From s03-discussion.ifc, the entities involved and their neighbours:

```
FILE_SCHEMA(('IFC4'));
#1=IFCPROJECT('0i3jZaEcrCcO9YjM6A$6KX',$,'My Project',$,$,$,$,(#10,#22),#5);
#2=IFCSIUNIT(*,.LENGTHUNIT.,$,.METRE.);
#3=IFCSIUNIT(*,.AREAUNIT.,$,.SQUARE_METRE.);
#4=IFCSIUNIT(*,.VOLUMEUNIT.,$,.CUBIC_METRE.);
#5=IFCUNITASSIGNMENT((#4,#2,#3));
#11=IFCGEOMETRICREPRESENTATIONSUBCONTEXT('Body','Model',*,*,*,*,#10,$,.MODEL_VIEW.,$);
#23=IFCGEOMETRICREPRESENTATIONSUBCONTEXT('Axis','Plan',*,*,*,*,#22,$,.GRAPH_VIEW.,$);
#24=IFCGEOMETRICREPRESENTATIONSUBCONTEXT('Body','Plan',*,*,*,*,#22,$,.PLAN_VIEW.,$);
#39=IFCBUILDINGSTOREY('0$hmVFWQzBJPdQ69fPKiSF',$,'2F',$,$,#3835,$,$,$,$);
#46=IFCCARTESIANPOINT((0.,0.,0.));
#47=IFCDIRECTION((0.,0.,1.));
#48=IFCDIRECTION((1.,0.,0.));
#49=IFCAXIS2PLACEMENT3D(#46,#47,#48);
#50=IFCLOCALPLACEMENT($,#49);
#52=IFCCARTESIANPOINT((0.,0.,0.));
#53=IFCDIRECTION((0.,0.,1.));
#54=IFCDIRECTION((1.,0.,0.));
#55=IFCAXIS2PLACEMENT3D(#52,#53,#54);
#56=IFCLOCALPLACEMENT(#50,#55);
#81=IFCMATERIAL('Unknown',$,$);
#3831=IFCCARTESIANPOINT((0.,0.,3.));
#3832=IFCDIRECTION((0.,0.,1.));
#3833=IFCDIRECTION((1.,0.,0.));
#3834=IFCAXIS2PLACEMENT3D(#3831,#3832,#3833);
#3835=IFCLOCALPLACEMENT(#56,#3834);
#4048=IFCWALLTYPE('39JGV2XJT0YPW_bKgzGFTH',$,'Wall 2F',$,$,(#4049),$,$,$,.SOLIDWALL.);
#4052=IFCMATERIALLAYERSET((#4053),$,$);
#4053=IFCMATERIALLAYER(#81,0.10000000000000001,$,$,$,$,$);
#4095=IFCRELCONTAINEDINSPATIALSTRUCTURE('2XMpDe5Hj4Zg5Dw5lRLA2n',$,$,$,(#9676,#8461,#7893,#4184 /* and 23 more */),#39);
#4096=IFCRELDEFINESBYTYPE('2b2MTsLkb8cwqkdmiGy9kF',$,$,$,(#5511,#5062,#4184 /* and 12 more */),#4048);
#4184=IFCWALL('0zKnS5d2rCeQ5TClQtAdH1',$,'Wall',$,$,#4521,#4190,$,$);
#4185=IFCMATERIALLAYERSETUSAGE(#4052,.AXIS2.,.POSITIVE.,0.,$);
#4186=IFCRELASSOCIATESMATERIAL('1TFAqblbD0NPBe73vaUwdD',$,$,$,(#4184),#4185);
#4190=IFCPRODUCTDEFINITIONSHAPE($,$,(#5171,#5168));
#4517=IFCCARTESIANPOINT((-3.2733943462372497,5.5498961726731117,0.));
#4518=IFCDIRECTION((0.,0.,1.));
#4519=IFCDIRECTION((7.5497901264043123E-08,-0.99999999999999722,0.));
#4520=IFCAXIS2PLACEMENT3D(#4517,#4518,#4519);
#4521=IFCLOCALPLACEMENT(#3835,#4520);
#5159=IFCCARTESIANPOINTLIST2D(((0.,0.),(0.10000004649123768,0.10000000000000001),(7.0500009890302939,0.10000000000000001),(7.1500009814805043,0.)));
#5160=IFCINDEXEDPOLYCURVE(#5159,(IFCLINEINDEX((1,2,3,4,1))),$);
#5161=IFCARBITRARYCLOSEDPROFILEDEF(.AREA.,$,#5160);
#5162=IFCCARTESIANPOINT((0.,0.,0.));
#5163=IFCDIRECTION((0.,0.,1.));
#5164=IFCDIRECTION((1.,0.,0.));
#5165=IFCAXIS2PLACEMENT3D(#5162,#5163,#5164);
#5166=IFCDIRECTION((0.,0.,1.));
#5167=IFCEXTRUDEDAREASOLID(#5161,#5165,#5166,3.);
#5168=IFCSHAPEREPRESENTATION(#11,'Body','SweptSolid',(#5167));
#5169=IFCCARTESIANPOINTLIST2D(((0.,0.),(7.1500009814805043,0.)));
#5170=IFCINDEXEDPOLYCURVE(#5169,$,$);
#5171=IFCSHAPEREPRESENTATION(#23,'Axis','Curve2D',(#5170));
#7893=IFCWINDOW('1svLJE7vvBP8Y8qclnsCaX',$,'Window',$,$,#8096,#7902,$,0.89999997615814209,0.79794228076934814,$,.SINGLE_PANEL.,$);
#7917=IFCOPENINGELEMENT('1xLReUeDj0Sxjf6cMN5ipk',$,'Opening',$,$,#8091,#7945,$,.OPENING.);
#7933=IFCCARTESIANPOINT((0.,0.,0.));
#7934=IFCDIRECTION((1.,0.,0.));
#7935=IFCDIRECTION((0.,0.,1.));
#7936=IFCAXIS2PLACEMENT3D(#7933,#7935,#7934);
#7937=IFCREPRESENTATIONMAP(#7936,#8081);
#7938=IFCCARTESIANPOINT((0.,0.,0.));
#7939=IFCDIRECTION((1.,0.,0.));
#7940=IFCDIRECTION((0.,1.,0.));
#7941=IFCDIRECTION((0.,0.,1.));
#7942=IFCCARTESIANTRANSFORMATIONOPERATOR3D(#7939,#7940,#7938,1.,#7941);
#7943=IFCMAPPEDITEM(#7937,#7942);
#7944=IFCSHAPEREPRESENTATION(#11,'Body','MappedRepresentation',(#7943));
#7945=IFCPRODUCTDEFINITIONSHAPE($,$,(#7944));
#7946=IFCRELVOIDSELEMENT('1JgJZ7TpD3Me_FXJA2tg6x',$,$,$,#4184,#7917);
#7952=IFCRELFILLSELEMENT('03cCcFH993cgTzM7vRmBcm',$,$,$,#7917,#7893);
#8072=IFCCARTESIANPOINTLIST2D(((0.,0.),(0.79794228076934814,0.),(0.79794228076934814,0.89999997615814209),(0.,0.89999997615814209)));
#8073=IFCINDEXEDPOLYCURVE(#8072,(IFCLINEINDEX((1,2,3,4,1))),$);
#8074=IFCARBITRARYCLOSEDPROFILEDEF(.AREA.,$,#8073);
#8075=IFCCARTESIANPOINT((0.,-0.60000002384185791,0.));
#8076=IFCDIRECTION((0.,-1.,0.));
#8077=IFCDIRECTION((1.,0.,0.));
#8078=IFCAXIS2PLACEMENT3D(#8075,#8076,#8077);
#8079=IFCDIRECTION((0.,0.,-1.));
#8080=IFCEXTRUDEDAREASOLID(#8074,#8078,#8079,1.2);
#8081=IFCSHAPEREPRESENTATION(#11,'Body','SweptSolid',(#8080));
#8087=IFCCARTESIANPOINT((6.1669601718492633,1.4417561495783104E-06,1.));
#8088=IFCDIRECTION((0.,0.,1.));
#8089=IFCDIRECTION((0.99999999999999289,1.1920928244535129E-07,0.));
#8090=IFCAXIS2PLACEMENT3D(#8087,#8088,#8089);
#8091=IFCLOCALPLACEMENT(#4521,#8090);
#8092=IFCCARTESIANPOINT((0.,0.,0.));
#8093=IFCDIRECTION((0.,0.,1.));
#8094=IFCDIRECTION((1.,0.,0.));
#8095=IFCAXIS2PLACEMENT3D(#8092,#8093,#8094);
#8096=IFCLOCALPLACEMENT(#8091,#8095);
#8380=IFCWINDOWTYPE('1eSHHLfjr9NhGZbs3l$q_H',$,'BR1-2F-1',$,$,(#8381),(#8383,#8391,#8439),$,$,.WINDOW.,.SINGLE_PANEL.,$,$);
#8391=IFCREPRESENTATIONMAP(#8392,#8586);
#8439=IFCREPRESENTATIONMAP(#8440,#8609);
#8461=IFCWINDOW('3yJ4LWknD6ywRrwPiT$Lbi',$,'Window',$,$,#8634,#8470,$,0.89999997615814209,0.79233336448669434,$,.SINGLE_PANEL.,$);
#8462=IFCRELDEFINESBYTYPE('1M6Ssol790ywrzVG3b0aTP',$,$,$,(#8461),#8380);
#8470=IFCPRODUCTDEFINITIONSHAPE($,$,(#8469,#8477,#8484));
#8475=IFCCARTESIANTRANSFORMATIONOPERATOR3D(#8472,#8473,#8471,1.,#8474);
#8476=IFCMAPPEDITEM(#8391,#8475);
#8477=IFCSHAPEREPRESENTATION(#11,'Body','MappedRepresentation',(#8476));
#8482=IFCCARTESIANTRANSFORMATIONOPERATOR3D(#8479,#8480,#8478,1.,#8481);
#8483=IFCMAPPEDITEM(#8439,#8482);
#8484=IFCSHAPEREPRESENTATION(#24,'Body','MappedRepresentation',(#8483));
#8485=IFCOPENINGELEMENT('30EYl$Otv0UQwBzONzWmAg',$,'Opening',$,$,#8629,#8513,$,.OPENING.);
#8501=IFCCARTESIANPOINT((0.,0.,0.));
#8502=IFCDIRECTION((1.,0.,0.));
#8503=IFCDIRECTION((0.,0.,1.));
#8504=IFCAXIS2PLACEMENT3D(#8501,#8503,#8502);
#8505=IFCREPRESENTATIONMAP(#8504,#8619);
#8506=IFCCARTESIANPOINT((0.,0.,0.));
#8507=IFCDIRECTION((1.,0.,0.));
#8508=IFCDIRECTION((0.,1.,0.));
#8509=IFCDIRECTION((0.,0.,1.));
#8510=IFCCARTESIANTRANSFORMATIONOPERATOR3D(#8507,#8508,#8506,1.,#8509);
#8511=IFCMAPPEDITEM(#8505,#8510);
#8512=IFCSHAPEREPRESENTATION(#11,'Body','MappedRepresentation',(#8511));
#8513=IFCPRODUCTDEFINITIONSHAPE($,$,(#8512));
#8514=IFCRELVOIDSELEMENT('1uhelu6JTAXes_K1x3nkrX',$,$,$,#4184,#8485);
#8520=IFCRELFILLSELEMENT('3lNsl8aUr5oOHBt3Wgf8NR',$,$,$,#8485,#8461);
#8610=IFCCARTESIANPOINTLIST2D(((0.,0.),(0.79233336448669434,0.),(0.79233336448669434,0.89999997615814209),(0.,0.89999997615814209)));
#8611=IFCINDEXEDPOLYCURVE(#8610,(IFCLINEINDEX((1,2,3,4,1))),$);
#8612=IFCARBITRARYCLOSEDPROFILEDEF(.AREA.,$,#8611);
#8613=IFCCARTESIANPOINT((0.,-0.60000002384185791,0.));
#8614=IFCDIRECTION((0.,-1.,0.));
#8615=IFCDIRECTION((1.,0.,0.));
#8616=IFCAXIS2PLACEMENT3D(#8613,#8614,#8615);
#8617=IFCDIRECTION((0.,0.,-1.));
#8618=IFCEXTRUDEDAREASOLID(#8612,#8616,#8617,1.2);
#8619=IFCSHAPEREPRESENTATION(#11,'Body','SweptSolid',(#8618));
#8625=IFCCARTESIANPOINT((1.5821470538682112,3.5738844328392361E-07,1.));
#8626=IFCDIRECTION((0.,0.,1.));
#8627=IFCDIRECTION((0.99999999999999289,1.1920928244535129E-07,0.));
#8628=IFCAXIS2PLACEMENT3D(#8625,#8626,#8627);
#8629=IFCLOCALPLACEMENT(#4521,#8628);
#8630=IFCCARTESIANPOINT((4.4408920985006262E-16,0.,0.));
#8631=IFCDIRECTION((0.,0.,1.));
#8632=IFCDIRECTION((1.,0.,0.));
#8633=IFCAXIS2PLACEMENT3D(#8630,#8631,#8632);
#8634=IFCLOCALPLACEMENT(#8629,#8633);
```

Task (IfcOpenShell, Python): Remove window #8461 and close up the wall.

```python
import ifcopenshell
import ifcopenshell.api.feature
import ifcopenshell.api.root
import ifcopenshell.geom
import ifcopenshell.util.shape

model = ifcopenshell.open("s03-discussion.ifc")
settings = ifcopenshell.geom.settings()


def volume(element):
    """Net volume in cubic metres, openings subtracted."""
    shape = ifcopenshell.geom.create_shape(settings, element)
    return ifcopenshell.util.shape.get_volume(shape.geometry)


window = model.by_guid("3yJ4LWknD6ywRrwPiT$Lbi")
opening = window.FillsVoids[0].RelatingOpeningElement
wall = opening.VoidsElements[0].RelatingBuildingElement
before = volume(wall)

ifcopenshell.api.root.remove_product(model, product=window)
ifcopenshell.api.feature.remove_feature(model, feature=opening)

after = volume(wall)

print(f"wall volume {before:.3f} -> {after:.3f} m3")

model.write("s03-discussion_edited.ifc")
```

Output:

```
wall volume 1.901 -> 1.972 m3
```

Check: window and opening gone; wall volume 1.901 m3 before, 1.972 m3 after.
